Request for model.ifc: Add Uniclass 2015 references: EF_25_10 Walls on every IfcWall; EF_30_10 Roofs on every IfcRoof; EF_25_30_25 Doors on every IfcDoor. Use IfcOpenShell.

First a look at what the model holds.

```python
import ifcopenshell

model = ifcopenshell.open("model.ifc")
print(model.schema)
print("classifications:", [c.Name for c in model.by_type("IfcClassification")])
for ifc_class in ("IfcDoor", "IfcRoof", "IfcStair", "IfcWall", "IfcWindow"):
    print(ifc_class, len(model.by_type(ifc_class)))
```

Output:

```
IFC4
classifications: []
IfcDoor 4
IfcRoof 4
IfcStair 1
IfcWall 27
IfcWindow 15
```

```python
import ifcopenshell
import ifcopenshell.api.classification

model = ifcopenshell.open("model.ifc")

system = ifcopenshell.api.classification.add_classification(model, classification="Uniclass 2015")

codes = {
    "IfcWall": ("EF_25_10", "Walls"),
    "IfcRoof": ("EF_30_10", "Roofs"),
    "IfcDoor": ("EF_25_30_25", "Doors"),
}
for ifc_class, (code, name) in codes.items():
    products = model.by_type(ifc_class)
    ifcopenshell.api.classification.add_reference(
        model, products=products, classification=system, identification=code, name=name
    )
    print(code, len(products))

model.write("model-out.ifc")
```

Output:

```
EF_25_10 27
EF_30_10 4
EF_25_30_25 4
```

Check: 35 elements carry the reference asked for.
